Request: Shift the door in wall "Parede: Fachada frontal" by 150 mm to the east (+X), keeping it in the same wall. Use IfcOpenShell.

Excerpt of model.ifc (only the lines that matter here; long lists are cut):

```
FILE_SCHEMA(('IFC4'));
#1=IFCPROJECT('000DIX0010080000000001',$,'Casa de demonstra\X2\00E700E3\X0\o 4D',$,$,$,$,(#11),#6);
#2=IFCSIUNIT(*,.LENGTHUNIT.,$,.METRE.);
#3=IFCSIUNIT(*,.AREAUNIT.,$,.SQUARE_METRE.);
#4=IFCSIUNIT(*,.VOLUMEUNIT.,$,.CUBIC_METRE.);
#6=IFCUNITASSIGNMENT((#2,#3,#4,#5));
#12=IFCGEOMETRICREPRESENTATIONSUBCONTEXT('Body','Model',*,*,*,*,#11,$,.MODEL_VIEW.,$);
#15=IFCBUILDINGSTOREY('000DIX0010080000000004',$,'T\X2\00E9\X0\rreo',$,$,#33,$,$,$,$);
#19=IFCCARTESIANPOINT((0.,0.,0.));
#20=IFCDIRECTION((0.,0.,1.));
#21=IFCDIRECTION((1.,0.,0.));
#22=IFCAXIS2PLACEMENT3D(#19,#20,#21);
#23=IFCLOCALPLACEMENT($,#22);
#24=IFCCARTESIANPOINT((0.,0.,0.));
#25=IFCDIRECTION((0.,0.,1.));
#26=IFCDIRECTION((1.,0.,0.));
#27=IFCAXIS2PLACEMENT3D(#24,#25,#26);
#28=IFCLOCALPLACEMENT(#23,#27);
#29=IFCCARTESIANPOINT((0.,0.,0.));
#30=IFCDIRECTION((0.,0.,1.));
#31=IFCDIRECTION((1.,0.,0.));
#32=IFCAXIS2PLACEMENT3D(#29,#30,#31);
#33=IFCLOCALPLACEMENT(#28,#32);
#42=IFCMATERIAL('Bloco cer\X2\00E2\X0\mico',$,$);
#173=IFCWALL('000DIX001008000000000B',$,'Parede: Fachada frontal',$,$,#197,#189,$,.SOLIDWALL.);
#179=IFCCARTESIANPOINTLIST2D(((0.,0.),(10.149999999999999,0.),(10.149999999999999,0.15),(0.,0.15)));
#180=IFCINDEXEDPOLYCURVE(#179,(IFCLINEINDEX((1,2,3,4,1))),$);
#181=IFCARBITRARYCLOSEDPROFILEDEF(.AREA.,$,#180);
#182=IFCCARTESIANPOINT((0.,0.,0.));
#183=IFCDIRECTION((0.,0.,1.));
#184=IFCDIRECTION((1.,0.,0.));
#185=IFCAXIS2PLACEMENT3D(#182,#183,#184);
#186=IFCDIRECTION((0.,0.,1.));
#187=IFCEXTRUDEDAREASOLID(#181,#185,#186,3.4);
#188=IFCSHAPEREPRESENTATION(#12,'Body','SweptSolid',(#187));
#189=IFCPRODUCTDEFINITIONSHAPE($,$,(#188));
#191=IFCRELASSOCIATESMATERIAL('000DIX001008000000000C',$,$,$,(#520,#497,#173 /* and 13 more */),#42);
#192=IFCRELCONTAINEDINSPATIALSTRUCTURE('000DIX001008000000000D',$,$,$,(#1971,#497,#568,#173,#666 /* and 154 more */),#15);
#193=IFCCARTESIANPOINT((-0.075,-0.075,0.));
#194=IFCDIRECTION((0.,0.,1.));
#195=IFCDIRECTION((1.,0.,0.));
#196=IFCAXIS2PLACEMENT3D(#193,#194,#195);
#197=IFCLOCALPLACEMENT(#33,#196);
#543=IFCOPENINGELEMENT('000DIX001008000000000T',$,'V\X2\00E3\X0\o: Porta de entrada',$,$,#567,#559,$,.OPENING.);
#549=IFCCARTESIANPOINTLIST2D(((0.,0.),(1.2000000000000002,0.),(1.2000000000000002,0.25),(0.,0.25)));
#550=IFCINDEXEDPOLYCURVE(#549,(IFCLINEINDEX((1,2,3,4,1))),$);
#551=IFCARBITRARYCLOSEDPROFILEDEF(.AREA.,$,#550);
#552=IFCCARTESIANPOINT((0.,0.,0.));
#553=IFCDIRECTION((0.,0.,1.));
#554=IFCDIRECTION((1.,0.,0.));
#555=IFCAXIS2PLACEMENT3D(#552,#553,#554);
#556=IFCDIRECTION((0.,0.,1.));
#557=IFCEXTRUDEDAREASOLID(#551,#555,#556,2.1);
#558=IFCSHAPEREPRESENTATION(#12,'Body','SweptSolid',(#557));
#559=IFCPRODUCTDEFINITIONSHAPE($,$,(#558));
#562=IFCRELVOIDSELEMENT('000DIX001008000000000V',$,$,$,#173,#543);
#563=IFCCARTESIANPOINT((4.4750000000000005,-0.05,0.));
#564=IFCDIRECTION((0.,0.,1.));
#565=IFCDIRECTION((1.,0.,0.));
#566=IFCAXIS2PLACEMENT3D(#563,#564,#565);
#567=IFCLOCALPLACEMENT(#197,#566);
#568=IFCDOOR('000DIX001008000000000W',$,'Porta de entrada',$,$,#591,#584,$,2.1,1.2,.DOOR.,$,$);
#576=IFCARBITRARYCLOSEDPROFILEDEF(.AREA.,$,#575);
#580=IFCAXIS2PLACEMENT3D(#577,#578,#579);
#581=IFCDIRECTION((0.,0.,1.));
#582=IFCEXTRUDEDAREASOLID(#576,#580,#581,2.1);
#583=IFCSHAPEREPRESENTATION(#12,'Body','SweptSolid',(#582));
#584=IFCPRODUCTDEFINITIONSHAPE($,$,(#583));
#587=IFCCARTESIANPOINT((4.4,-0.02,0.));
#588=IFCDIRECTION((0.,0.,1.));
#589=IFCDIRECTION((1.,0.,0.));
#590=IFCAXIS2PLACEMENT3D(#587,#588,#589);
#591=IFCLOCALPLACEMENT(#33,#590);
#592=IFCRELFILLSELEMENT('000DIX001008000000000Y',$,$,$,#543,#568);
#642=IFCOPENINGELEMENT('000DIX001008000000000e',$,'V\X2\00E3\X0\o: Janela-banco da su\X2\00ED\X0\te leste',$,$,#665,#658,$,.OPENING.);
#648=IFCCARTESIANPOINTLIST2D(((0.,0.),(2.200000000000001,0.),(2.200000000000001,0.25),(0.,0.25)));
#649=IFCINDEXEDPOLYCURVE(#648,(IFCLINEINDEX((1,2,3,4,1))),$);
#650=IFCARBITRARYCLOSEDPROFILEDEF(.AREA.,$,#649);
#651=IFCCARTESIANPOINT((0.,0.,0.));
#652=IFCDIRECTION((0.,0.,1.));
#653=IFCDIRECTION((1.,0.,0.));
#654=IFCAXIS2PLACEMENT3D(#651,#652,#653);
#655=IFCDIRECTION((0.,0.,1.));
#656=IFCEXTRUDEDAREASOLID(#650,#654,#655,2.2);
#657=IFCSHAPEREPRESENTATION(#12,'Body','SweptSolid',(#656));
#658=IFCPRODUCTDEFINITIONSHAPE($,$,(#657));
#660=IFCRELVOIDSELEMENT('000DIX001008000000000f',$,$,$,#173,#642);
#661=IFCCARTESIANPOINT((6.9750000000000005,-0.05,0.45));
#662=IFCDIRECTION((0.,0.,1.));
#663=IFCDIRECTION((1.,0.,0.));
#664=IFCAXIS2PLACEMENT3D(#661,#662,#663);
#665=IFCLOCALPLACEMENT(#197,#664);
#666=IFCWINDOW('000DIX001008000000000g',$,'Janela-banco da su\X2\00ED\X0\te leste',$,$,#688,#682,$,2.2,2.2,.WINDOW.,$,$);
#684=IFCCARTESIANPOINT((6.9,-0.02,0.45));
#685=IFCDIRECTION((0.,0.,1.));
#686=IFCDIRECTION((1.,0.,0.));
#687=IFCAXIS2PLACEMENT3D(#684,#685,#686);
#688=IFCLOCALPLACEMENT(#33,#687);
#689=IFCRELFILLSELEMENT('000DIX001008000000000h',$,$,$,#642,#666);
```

```python
import ifcopenshell
import ifcopenshell.api.geometry
import ifcopenshell.util.placement

model = ifcopenshell.open("model.ifc")

door = model.by_guid("000DIX001008000000000W")
opening = door.FillsVoids[0].RelatingOpeningElement
wall = opening.VoidsElements[0].RelatingBuildingElement

wall_matrix = ifcopenshell.util.placement.get_local_placement(wall.ObjectPlacement)
shift = wall_matrix[:3, 0] * 0.15
before = ifcopenshell.util.placement.get_local_placement(door.ObjectPlacement)[:3, 3].copy()

# The door is not placed relative to its opening, so move both.
for product in (opening, door):
    matrix = ifcopenshell.util.placement.get_local_placement(product.ObjectPlacement)
    matrix[:3, 3] += shift
    ifcopenshell.api.geometry.edit_object_placement(model, product=product, matrix=matrix, is_si=False)

after = ifcopenshell.util.placement.get_local_placement(door.ObjectPlacement)[:3, 3]
print("door moved by", (after - before).round(3) + 0.0)

model.write("model_v2.ifc")
```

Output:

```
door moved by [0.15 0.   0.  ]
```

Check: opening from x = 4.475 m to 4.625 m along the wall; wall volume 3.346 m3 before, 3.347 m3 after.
